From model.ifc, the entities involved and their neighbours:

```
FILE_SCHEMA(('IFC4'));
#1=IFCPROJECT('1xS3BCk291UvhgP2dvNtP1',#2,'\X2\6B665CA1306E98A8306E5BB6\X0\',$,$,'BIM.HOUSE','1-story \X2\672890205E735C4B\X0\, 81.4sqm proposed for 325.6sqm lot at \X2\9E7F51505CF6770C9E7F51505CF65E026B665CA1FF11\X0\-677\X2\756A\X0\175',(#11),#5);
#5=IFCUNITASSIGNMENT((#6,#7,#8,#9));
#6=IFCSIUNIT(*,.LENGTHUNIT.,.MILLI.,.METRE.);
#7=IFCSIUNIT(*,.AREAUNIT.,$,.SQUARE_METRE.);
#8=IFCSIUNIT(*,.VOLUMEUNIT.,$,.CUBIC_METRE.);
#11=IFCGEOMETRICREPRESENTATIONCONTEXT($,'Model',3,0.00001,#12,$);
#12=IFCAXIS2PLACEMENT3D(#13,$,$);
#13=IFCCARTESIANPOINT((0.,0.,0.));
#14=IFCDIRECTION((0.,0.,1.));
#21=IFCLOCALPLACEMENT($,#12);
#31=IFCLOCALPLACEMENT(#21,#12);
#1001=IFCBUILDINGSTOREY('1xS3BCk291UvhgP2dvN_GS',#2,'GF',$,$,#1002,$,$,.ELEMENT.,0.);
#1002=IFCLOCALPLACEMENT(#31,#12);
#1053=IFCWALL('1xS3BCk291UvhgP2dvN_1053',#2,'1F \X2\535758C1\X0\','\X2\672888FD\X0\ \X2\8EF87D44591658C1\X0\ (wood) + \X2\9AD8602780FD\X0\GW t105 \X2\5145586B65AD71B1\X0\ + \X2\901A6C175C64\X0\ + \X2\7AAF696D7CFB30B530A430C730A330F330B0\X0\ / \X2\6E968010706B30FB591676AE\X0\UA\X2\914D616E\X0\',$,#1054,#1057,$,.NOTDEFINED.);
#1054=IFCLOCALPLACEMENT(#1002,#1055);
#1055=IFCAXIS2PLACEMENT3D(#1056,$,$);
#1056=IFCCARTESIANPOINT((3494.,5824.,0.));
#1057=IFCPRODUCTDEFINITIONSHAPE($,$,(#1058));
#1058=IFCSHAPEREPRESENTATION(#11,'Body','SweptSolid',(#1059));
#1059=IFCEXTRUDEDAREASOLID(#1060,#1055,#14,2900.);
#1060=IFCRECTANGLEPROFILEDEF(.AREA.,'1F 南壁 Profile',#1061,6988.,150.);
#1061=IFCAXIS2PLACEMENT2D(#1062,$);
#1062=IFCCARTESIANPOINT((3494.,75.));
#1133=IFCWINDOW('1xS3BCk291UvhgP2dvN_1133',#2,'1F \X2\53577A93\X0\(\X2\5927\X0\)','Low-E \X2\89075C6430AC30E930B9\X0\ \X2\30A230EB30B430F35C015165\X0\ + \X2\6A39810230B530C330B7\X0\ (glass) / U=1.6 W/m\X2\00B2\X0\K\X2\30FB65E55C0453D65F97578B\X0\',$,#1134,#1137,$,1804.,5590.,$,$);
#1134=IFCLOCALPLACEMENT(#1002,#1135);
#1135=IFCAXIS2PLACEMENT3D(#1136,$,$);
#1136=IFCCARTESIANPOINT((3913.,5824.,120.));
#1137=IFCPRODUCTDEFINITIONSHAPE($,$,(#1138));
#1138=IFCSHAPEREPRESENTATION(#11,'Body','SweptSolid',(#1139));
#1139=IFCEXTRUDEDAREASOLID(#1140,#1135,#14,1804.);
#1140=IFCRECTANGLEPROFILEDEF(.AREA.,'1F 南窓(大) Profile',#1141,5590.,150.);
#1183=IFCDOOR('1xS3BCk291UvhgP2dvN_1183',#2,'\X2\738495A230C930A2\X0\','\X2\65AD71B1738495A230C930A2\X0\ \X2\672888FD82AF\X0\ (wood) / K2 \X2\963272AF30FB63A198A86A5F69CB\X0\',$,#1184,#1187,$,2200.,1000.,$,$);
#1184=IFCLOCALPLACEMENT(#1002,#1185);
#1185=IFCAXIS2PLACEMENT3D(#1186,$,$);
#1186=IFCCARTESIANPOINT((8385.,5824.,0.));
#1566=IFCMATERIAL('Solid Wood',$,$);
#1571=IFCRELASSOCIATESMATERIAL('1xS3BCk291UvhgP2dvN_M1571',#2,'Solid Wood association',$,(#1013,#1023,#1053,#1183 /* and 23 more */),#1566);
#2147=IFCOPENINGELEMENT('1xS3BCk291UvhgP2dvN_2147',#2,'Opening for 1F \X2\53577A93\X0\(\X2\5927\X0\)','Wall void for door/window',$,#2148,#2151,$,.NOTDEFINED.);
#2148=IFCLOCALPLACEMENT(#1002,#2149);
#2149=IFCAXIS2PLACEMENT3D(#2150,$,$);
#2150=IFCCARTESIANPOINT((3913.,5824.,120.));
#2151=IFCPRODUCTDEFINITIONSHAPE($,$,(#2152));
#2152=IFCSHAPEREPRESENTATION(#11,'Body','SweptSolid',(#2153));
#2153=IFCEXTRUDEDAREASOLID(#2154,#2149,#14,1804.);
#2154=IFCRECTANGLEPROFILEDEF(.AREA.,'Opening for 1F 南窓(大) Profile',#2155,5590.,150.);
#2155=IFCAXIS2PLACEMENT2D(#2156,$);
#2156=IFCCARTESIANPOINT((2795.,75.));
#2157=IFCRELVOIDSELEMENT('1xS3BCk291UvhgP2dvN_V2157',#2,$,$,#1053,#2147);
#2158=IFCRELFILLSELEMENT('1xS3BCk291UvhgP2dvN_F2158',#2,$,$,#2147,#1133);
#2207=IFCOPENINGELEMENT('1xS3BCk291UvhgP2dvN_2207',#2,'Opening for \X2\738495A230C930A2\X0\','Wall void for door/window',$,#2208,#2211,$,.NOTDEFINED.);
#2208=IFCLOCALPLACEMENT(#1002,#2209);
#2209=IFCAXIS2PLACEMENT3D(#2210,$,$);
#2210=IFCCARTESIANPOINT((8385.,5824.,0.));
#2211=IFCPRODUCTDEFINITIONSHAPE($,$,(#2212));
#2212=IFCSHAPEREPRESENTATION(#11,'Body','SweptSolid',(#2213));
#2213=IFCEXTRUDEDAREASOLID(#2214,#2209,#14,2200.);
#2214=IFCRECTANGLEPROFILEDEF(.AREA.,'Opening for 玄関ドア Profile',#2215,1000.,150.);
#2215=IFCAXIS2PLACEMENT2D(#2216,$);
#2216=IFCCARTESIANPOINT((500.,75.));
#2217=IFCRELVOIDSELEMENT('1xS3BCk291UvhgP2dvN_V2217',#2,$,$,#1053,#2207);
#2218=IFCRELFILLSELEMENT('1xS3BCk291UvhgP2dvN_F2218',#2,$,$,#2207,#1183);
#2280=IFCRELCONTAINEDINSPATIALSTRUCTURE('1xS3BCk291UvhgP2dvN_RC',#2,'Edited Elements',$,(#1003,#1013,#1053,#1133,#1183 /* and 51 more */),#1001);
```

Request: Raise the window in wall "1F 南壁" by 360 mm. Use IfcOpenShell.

```python
import numpy as np
import ifcopenshell
import ifcopenshell.api.geometry
import ifcopenshell.util.placement
import ifcopenshell.util.unit

model = ifcopenshell.open("model.ifc")
unit_scale = ifcopenshell.util.unit.calculate_unit_scale(model)

window = model.by_id(1133)
opening = window.FillsVoids[0].RelatingOpeningElement
dz = 0.36 / unit_scale

shift = np.array([0.0, 0.0, dz])
# The window is not placed relative to its opening, so move both.
for product in (opening, window):
    matrix = ifcopenshell.util.placement.get_local_placement(product.ObjectPlacement)
    matrix[:3, 3] += shift
    ifcopenshell.api.geometry.edit_object_placement(model, product=product, matrix=matrix, is_si=False)

print(f"moved by {dz * unit_scale:+.3f} m")

model.write("model_edited.ifc")
```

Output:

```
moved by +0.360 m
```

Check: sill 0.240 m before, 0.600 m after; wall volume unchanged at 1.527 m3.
